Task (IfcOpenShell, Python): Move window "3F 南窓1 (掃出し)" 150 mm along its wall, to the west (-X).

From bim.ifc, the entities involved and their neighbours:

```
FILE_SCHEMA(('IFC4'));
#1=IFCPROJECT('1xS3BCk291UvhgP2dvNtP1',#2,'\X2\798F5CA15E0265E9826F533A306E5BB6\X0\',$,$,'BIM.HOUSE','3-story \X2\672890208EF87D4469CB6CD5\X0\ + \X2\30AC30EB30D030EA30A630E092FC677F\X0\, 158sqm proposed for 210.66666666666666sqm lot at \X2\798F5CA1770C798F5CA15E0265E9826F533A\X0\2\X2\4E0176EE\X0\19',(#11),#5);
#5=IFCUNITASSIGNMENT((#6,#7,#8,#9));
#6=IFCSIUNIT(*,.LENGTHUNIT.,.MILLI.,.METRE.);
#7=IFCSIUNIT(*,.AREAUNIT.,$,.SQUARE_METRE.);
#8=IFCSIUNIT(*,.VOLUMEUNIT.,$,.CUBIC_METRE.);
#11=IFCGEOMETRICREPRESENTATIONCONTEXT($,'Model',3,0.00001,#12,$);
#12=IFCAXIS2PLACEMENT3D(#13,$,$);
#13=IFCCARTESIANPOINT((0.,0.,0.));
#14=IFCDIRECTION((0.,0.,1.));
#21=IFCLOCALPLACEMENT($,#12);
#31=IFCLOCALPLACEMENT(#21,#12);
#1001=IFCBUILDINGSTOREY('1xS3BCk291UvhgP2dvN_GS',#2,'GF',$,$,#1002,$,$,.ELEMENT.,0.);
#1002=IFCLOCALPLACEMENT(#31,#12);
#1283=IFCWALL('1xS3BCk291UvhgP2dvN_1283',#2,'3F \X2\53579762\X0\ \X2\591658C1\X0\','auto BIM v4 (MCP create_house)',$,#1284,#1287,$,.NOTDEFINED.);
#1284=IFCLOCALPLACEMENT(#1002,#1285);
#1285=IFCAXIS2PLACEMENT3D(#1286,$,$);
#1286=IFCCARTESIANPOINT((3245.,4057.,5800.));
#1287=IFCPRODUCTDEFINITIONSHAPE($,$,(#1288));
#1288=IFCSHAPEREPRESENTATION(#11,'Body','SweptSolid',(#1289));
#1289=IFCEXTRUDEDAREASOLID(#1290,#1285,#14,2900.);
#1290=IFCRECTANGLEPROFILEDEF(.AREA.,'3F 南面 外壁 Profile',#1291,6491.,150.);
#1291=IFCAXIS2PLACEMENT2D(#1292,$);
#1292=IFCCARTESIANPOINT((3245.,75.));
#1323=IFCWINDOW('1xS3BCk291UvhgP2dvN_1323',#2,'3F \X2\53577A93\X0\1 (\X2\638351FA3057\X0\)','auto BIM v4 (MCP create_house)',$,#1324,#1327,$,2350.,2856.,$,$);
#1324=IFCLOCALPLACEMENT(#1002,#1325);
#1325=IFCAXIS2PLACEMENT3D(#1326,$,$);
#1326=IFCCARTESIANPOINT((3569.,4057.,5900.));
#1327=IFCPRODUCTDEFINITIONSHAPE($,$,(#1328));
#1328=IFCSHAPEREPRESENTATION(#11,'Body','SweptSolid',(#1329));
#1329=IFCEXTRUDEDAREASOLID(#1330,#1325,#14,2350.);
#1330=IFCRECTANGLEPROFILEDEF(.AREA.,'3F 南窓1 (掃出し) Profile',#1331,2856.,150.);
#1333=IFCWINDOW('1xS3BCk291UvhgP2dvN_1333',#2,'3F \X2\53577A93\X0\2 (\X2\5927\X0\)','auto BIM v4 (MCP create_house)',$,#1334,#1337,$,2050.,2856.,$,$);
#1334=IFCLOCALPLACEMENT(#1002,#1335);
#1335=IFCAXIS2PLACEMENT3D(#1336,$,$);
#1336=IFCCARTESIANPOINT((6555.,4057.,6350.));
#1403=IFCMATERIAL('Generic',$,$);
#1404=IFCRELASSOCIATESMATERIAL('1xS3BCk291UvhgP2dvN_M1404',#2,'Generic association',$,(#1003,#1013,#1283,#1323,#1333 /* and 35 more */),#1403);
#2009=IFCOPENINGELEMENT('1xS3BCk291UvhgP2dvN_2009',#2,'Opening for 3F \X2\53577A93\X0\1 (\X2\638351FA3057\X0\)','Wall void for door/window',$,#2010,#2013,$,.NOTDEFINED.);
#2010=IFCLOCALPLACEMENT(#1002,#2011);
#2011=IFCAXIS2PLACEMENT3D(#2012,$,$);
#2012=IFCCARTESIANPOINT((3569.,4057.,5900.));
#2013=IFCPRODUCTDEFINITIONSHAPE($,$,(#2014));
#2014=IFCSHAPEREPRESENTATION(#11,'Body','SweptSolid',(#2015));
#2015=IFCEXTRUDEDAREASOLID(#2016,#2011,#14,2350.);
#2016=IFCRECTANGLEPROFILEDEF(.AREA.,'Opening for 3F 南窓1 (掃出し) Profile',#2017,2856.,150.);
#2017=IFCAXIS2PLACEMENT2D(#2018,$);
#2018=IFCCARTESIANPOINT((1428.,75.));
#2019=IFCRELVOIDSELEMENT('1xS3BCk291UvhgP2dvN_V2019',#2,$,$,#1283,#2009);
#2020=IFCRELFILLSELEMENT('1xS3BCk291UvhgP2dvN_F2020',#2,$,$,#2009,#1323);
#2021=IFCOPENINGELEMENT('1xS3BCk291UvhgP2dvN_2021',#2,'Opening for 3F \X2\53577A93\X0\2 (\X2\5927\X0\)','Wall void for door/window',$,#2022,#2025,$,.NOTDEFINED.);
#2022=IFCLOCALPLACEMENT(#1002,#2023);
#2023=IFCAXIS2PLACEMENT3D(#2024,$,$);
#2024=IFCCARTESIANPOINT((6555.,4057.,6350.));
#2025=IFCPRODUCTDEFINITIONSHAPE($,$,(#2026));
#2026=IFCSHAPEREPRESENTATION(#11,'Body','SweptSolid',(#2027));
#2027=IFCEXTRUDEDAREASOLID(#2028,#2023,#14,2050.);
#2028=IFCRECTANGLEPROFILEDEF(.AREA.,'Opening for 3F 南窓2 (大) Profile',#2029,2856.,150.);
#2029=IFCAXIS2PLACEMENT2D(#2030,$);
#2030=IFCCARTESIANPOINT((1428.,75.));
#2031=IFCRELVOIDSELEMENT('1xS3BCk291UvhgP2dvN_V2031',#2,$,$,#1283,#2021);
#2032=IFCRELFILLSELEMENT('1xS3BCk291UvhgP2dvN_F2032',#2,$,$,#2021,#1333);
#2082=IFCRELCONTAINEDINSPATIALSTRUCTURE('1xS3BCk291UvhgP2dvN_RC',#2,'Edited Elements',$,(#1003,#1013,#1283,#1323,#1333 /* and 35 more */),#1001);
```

```python
import ifcopenshell
import ifcopenshell.api.geometry
import ifcopenshell.util.placement

model = ifcopenshell.open("bim.ifc")

window = model.by_guid("1xS3BCk291UvhgP2dvN_1323")
opening = window.FillsVoids[0].RelatingOpeningElement
wall = opening.VoidsElements[0].RelatingBuildingElement

wall_matrix = ifcopenshell.util.placement.get_local_placement(wall.ObjectPlacement)
shift = wall_matrix[:3, 0] * -150.0
before = ifcopenshell.util.placement.get_local_placement(window.ObjectPlacement)[:3, 3].copy()

# The window is not placed relative to its opening, so move both.
for product in (opening, window):
    matrix = ifcopenshell.util.placement.get_local_placement(product.ObjectPlacement)
    matrix[:3, 3] += shift
    ifcopenshell.api.geometry.edit_object_placement(model, product=product, matrix=matrix, is_si=False)

after = ifcopenshell.util.placement.get_local_placement(window.ObjectPlacement)[:3, 3]
print("window moved by", (after - before).round(3) + 0.0)

model.write("bim_v2.ifc")
```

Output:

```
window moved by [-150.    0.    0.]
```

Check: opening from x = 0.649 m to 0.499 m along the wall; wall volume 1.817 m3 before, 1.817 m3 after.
